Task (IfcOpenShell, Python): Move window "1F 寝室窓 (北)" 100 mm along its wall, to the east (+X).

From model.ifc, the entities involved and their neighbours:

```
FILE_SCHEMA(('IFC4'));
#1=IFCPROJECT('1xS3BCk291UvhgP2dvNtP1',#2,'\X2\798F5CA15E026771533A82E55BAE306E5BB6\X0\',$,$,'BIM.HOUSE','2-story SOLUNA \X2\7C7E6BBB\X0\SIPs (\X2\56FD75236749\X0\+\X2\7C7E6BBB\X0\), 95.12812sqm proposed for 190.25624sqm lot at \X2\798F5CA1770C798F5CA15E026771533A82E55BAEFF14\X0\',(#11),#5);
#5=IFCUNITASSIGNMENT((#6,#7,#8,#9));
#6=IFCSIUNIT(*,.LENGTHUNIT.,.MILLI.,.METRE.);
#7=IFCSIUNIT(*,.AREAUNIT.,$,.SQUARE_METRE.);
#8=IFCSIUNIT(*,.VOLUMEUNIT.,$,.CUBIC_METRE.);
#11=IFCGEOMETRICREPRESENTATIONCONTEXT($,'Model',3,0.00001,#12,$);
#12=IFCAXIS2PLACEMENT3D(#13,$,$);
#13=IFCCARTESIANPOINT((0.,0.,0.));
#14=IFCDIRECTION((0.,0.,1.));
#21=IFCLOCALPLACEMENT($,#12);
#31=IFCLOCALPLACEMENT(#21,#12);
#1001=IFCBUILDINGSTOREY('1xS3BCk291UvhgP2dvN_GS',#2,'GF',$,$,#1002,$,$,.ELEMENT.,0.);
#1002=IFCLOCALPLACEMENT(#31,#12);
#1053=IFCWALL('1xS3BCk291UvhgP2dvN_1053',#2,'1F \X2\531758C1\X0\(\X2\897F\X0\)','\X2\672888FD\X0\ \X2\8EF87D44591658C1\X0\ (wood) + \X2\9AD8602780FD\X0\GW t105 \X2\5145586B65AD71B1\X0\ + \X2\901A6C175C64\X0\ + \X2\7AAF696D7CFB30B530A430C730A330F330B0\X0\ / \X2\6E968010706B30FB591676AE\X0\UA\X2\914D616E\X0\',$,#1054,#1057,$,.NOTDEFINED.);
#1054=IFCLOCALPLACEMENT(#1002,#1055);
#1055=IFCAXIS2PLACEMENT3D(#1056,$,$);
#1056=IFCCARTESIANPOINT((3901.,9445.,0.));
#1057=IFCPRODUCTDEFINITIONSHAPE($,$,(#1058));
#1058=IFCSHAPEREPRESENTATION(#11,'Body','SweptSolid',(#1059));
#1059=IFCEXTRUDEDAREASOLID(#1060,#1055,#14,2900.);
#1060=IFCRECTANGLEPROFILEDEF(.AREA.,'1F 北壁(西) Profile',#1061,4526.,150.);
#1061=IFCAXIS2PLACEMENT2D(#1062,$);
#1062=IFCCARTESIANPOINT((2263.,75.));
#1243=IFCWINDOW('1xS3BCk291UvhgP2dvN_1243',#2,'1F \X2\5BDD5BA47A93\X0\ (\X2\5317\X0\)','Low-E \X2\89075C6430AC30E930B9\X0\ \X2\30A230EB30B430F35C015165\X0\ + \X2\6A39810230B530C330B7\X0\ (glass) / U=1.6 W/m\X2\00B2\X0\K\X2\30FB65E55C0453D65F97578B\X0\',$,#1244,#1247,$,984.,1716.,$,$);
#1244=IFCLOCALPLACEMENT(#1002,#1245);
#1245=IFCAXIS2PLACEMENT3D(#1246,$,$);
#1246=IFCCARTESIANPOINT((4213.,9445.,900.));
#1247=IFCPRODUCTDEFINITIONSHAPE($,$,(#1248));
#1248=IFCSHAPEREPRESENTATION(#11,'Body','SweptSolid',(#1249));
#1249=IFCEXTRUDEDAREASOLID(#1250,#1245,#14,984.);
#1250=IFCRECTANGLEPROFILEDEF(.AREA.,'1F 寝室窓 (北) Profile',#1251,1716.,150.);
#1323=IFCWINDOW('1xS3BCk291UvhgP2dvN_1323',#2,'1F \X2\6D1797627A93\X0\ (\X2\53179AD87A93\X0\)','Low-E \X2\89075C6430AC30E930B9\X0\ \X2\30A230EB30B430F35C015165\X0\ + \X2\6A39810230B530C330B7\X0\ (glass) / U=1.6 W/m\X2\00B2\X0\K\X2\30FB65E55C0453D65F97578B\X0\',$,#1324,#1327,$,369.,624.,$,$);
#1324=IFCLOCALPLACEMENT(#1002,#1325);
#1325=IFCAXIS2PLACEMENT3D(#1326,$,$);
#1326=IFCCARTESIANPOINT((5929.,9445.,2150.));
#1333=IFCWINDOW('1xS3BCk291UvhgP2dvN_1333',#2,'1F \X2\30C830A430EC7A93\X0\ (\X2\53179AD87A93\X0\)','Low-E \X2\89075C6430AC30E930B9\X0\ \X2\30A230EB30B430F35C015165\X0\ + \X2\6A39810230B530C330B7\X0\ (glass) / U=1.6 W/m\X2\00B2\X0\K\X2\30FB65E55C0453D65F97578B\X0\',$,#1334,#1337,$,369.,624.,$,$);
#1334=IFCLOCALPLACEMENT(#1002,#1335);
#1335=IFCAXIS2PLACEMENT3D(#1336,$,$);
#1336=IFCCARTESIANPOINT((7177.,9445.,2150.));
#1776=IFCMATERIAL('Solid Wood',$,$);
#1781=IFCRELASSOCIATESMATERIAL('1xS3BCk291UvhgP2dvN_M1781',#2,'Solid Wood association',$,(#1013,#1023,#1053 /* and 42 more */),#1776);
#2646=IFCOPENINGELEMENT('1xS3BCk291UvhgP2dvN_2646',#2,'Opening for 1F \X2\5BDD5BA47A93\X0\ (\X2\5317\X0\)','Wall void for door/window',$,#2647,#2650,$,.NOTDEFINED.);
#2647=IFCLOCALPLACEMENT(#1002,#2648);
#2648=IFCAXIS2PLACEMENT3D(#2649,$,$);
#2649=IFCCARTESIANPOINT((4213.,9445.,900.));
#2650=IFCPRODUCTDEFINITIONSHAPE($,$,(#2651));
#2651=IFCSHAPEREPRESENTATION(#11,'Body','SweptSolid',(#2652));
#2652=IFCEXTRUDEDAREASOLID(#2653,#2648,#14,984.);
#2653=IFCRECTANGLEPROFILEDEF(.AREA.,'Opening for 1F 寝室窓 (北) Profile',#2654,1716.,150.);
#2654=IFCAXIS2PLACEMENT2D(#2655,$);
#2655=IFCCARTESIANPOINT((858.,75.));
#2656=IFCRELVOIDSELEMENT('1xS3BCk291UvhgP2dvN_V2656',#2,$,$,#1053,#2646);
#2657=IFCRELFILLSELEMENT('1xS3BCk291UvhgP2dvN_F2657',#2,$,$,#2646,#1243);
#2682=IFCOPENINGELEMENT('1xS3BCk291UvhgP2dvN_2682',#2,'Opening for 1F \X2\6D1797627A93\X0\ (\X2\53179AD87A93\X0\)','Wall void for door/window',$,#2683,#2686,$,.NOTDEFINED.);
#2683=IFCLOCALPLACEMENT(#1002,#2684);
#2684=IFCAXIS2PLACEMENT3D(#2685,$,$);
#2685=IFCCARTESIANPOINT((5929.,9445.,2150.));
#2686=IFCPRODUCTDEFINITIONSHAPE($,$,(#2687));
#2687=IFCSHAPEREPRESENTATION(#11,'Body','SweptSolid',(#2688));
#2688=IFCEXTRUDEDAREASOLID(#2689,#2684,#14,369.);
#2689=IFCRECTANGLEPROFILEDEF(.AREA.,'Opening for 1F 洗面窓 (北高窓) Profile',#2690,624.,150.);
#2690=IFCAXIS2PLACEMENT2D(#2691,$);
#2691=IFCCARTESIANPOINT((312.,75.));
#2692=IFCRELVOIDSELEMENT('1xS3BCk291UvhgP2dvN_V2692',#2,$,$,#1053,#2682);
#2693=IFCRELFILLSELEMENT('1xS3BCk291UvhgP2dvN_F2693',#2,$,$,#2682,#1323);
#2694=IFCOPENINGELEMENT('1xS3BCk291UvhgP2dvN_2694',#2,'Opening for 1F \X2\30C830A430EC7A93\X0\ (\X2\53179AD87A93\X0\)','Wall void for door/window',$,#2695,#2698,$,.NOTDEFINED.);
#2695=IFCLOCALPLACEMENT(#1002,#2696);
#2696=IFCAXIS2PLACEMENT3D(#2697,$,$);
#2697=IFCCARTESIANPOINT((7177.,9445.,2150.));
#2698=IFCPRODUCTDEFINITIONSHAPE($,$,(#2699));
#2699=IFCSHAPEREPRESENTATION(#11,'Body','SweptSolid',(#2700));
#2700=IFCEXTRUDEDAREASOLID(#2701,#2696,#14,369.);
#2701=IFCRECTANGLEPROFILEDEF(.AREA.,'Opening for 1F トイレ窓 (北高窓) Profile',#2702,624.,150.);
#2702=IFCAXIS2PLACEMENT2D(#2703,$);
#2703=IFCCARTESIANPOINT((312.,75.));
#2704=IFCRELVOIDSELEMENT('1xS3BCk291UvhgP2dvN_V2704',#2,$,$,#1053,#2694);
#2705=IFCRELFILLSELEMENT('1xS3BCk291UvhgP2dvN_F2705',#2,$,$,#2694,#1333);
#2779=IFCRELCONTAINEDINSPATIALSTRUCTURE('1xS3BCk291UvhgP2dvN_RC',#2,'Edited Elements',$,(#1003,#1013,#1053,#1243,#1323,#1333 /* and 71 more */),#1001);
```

```python
import ifcopenshell
import ifcopenshell.api.geometry
import ifcopenshell.util.placement
import ifcopenshell.util.unit

model = ifcopenshell.open("model.ifc")
unit_scale = ifcopenshell.util.unit.calculate_unit_scale(model)

window = model.by_id(1243)
opening = window.FillsVoids[0].RelatingOpeningElement
wall = opening.VoidsElements[0].RelatingBuildingElement

wall_matrix = ifcopenshell.util.placement.get_local_placement(wall.ObjectPlacement)
shift = wall_matrix[:3, 0] * 0.1 / unit_scale
before = ifcopenshell.util.placement.get_local_placement(window.ObjectPlacement)[:3, 3].copy()

# The window is not placed relative to its opening, so move both.
for product in (opening, window):
    matrix = ifcopenshell.util.placement.get_local_placement(product.ObjectPlacement)
    matrix[:3, 3] += shift
    ifcopenshell.api.geometry.edit_object_placement(model, product=product, matrix=matrix, is_si=False)

after = ifcopenshell.util.placement.get_local_placement(window.ObjectPlacement)[:3, 3]
print("window moved by", (after - before).round(3) + 0.0)

model.write("model-out.ifc")
```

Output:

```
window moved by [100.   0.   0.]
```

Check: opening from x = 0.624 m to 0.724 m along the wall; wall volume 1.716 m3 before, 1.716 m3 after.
